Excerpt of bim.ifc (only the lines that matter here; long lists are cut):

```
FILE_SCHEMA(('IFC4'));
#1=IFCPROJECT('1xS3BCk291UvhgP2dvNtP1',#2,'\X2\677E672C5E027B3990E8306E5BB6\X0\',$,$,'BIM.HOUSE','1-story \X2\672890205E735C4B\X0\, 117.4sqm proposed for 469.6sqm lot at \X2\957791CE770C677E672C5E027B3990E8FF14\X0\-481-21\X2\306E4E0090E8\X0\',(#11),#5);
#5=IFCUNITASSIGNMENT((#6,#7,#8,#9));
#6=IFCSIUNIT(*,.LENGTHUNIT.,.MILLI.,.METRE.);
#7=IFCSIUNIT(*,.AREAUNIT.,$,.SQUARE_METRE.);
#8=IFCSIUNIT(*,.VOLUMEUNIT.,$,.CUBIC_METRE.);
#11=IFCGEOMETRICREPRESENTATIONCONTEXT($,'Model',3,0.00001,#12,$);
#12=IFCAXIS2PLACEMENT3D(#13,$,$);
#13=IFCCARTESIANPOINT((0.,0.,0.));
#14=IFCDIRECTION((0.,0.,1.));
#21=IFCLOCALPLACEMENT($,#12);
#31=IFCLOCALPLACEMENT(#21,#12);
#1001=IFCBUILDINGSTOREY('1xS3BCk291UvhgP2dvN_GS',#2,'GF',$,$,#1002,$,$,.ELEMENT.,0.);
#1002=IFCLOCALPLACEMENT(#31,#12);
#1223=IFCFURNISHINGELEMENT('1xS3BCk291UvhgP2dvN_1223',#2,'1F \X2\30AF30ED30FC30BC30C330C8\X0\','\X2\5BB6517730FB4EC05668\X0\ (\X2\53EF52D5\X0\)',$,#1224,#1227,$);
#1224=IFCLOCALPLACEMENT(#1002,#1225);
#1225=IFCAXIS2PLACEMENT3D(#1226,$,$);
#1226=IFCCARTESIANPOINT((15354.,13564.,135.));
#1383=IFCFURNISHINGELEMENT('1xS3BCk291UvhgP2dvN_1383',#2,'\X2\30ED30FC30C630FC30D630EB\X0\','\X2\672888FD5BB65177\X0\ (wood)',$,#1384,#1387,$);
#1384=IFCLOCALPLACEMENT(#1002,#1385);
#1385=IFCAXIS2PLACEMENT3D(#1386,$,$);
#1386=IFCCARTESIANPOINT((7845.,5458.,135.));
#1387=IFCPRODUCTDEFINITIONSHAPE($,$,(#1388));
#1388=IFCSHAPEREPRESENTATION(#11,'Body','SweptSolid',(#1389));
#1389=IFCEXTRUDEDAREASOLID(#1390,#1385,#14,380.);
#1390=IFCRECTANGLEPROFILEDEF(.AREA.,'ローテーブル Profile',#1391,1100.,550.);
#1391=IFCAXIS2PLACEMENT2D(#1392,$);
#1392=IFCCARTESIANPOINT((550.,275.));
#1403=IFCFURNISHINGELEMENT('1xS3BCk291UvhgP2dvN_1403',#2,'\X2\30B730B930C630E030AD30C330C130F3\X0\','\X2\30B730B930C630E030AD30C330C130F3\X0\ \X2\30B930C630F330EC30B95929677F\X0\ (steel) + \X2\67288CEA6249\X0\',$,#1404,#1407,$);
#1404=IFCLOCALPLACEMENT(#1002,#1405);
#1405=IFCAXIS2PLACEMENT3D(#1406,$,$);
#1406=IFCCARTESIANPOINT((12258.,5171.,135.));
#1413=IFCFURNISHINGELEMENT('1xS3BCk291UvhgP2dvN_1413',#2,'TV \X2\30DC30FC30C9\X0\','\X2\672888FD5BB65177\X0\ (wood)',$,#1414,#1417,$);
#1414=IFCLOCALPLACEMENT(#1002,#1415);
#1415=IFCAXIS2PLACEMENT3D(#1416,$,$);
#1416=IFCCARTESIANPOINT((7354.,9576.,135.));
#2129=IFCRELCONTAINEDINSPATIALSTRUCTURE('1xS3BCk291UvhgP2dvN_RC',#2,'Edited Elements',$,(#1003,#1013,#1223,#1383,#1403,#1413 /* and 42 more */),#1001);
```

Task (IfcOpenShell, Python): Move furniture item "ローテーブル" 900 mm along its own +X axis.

```python
import ifcopenshell
import ifcopenshell.api.geometry
import ifcopenshell.util.placement
import ifcopenshell.util.unit

model = ifcopenshell.open("bim.ifc")
unit_scale = ifcopenshell.util.unit.calculate_unit_scale(model)

item = model.by_id(1383)
matrix = ifcopenshell.util.placement.get_local_placement(item.ObjectPlacement)
matrix[:3, 3] += matrix[:3, 0] * 0.9 / unit_scale
ifcopenshell.api.geometry.edit_object_placement(model, product=item, matrix=matrix, is_si=False)

print(ifcopenshell.util.placement.get_local_placement(item.ObjectPlacement).round(3) + 0.0)

model.write("bim-out.ifc")
```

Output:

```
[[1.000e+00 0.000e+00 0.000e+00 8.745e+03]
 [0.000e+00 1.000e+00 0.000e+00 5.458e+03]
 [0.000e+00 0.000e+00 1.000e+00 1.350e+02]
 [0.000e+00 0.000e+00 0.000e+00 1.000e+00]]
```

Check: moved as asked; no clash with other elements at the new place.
